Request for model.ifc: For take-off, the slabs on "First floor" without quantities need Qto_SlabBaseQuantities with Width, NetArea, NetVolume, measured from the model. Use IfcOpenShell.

First a look at what the model holds.

```python
import ifcopenshell
import ifcopenshell.util.element
import ifcopenshell.util.unit

model = ifcopenshell.open("model.ifc")
print(model.schema)
for unit_type in ("LENGTHUNIT", "AREAUNIT", "VOLUMEUNIT"):
    print(unit_type, ifcopenshell.util.unit.calculate_unit_scale(model, unit_type))
storey = next(s for s in model.by_type("IfcBuildingStorey") if s.Name == "First floor")
slabs = [e for e in ifcopenshell.util.element.get_decomposition(storey) if e.is_a("IfcSlab")]
for e in sorted(slabs, key=lambda e: e.id()):
    print(e.id(), e.is_a(), e.Name, list(ifcopenshell.util.element.get_psets(e, qtos_only=True)), sep=" | ")
```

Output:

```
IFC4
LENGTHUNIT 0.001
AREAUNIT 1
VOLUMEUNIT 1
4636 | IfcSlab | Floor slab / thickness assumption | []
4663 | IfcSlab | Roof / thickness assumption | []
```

```python
import ifcopenshell
import ifcopenshell.api.pset
import ifcopenshell.geom
import ifcopenshell.util.element
import ifcopenshell.util.shape
import ifcopenshell.util.unit

model = ifcopenshell.open("model.ifc")
unit_scale = ifcopenshell.util.unit.calculate_unit_scale(model)
area_scale = ifcopenshell.util.unit.calculate_unit_scale(model, "AREAUNIT")
volume_scale = ifcopenshell.util.unit.calculate_unit_scale(model, "VOLUMEUNIT")
settings = ifcopenshell.geom.settings()

storey = next(s for s in model.by_type("IfcBuildingStorey") if s.Name == "First floor")
slabs = [e for e in ifcopenshell.util.element.get_decomposition(storey) if e.is_a("IfcSlab")]

for e in sorted(slabs, key=lambda e: e.id()):
    if ifcopenshell.util.element.get_psets(e, qtos_only=True, should_inherit=False):
        continue
    # Geometry comes back in metres, in the element's own axes.
    shape = ifcopenshell.geom.create_shape(settings, e)
    values = {
        "Width": ifcopenshell.util.shape.get_z(shape.geometry) / unit_scale,
        "NetArea": ifcopenshell.util.shape.get_footprint_area(shape.geometry) / area_scale,
        "NetVolume": ifcopenshell.util.shape.get_volume(shape.geometry) / volume_scale,
    }
    qto = ifcopenshell.api.pset.add_qto(model, product=e, name="Qto_SlabBaseQuantities")
    ifcopenshell.api.pset.edit_qto(model, qto=qto, properties=values)
    print(e.id(), {k: round(v, 3) for k, v in values.items()})

model.write("model_updated.ifc")
```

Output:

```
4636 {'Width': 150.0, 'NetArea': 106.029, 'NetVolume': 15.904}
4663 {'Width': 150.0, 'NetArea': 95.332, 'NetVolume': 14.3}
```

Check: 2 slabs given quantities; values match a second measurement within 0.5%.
